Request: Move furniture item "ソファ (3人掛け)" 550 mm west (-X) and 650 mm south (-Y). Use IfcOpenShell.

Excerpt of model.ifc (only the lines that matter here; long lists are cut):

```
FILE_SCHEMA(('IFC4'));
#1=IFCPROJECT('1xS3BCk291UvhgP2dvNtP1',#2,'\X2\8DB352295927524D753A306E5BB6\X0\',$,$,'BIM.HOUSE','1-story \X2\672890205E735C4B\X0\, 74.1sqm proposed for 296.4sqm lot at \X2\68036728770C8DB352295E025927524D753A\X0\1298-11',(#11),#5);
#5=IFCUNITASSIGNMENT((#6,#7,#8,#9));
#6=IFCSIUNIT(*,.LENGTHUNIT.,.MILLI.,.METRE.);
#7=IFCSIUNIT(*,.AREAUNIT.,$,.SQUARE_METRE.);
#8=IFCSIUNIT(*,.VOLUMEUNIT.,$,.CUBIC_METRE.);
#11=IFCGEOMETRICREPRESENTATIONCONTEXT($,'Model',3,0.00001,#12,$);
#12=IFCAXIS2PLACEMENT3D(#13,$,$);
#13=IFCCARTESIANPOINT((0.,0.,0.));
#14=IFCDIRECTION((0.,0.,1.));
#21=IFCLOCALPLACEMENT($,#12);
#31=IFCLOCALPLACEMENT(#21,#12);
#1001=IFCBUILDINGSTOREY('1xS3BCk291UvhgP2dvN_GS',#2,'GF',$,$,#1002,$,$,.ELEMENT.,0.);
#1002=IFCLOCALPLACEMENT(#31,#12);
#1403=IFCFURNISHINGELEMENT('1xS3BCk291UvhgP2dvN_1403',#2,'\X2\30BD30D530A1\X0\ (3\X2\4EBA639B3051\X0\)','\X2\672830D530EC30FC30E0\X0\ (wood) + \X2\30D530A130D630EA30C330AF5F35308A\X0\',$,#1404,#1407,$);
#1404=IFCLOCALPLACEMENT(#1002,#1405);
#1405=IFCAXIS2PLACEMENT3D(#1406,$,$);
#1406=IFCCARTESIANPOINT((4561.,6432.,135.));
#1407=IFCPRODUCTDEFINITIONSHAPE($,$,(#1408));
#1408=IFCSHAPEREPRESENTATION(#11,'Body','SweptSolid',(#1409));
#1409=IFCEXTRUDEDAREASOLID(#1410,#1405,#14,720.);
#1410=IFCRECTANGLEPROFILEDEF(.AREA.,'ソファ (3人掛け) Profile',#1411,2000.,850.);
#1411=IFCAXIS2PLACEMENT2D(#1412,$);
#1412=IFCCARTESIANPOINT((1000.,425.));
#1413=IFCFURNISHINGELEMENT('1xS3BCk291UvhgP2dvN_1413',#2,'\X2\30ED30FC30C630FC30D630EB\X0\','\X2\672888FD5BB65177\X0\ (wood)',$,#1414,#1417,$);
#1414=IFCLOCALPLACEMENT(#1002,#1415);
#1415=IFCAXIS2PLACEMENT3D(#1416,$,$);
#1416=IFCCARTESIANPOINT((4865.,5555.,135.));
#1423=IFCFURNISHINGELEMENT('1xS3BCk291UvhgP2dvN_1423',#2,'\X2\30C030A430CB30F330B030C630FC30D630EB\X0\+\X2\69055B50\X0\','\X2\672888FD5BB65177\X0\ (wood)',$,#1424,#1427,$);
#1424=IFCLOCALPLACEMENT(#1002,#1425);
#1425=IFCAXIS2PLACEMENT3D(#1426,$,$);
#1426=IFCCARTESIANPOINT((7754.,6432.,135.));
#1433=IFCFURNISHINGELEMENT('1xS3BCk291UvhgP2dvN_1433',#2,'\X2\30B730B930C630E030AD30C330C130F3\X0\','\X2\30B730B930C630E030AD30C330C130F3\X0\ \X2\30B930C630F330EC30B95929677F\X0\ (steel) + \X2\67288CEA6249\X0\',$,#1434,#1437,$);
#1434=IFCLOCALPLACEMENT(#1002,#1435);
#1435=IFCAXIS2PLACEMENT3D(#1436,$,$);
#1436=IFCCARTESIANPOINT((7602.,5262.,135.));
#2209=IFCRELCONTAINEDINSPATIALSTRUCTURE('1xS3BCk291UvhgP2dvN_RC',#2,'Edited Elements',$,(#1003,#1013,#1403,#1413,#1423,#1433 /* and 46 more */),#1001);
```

```python
import ifcopenshell
import ifcopenshell.api.geometry
import ifcopenshell.util.placement
import ifcopenshell.util.unit

model = ifcopenshell.open("model.ifc")
unit_scale = ifcopenshell.util.unit.calculate_unit_scale(model)

item = model.by_id(1403)
matrix = ifcopenshell.util.placement.get_local_placement(item.ObjectPlacement)
matrix[0, 3] -= 0.55 / unit_scale
matrix[1, 3] -= 0.65 / unit_scale
ifcopenshell.api.geometry.edit_object_placement(model, product=item, matrix=matrix, is_si=False)

print(ifcopenshell.util.placement.get_local_placement(item.ObjectPlacement).round(3) + 0.0)

model.write("model_v2.ifc")
```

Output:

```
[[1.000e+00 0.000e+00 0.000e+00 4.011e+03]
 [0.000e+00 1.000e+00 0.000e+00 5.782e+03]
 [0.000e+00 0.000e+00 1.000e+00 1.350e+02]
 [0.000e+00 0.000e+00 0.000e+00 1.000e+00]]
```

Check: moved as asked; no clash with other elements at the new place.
